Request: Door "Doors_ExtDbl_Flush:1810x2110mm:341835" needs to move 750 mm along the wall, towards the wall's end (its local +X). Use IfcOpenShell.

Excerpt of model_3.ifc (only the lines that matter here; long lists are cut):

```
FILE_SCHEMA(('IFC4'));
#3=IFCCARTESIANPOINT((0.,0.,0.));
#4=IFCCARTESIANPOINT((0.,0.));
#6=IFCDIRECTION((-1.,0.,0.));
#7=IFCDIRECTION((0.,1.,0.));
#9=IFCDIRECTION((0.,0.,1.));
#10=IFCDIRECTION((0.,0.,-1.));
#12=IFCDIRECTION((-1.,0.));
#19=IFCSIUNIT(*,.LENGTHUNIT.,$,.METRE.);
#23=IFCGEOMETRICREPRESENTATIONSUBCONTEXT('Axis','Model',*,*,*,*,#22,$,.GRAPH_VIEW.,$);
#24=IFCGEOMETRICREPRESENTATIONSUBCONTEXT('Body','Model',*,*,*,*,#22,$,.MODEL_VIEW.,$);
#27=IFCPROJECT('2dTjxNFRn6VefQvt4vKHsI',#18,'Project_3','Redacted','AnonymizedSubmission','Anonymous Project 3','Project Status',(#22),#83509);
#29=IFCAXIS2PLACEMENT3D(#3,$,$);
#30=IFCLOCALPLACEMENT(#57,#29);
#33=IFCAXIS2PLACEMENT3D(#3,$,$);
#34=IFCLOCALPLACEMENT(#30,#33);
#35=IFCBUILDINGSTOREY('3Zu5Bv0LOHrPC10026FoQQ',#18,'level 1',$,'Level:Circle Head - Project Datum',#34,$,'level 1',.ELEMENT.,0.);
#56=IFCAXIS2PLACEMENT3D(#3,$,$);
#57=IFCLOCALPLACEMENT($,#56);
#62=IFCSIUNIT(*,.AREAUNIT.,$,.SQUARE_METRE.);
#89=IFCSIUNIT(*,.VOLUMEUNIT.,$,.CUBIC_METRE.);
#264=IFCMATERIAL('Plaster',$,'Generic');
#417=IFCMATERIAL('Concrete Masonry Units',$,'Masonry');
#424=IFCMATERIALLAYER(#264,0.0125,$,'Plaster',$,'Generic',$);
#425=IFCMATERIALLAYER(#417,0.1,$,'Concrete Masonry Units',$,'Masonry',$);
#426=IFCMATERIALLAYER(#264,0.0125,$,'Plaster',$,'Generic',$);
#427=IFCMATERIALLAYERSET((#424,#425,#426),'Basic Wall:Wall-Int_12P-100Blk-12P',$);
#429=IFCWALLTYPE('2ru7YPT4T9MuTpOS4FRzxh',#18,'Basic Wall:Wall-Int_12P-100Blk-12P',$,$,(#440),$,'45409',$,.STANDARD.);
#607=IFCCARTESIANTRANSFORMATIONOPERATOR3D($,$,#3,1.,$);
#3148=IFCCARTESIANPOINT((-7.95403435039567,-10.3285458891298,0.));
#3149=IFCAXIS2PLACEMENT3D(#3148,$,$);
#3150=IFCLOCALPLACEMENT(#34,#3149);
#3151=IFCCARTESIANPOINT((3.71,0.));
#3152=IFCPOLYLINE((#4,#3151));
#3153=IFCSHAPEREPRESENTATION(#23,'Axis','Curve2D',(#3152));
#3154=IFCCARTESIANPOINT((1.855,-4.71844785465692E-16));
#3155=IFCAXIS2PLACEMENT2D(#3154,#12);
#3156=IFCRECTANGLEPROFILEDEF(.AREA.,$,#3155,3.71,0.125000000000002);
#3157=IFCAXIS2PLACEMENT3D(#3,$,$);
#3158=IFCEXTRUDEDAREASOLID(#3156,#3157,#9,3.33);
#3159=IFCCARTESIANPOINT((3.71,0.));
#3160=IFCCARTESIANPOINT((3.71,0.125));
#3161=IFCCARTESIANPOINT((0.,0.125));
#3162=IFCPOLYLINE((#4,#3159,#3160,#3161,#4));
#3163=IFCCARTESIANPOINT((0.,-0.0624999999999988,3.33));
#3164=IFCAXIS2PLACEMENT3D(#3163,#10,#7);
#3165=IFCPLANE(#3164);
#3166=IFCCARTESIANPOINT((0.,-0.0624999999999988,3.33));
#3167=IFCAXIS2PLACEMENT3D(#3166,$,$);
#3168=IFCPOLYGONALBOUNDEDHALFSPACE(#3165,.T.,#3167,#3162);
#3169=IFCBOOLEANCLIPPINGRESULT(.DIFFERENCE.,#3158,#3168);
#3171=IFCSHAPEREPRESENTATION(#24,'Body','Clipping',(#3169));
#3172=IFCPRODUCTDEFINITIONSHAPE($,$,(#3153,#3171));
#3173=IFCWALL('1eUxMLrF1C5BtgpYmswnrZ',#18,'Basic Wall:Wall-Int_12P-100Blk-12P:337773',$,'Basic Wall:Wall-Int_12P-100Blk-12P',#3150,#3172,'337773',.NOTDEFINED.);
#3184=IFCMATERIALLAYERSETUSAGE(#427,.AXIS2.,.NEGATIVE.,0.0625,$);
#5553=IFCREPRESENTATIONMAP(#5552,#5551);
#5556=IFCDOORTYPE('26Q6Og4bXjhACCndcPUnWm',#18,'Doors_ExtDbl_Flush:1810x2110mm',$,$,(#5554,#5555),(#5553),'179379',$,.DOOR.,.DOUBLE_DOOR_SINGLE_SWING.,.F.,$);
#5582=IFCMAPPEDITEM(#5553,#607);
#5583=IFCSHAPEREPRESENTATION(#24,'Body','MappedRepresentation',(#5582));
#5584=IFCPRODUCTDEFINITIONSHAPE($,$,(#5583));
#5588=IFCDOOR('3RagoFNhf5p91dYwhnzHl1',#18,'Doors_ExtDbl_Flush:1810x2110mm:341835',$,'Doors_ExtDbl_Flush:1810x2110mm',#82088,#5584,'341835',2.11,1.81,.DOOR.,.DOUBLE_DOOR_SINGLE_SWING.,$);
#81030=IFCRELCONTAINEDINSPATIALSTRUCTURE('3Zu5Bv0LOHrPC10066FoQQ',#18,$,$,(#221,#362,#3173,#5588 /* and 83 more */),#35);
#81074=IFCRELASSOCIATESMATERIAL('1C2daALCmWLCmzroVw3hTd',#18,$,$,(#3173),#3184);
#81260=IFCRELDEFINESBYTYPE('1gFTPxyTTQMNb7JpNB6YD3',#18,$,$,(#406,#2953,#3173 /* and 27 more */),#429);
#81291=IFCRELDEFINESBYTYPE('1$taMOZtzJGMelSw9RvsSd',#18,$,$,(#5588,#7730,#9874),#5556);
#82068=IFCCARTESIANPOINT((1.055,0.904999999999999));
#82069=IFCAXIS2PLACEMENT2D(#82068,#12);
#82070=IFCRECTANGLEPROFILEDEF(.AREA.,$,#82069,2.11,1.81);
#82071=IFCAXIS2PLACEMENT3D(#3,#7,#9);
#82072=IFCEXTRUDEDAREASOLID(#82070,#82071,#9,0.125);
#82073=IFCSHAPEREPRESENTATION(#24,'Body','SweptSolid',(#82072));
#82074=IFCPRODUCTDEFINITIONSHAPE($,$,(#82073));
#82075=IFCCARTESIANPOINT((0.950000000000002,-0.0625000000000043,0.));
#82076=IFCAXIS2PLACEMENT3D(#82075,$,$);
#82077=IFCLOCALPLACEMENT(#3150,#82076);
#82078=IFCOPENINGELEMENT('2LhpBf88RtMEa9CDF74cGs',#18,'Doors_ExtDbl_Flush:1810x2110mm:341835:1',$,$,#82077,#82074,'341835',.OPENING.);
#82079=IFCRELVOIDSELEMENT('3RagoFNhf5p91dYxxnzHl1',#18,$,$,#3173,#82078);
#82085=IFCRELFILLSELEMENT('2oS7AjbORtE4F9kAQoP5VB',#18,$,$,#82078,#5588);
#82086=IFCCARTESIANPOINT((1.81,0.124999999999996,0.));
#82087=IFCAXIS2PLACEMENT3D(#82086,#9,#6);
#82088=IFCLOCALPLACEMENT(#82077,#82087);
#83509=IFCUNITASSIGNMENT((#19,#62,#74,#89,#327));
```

```python
import ifcopenshell
import ifcopenshell.api.geometry
import ifcopenshell.util.placement
import ifcopenshell.util.unit

model = ifcopenshell.open("model_3.ifc")
unit_scale = ifcopenshell.util.unit.calculate_unit_scale(model)

door = model.by_guid("3RagoFNhf5p91dYwhnzHl1")
opening = door.FillsVoids[0].RelatingOpeningElement
wall = opening.VoidsElements[0].RelatingBuildingElement

wall_matrix = ifcopenshell.util.placement.get_local_placement(wall.ObjectPlacement)
shift = wall_matrix[:3, 0] * 0.75 / unit_scale
before = ifcopenshell.util.placement.get_local_placement(door.ObjectPlacement)[:3, 3].copy()

# The door is placed relative to its opening, so it follows when the opening moves.
matrix = ifcopenshell.util.placement.get_local_placement(opening.ObjectPlacement)
matrix[:3, 3] += shift
ifcopenshell.api.geometry.edit_object_placement(
    model, product=opening, matrix=matrix, is_si=False, should_transform_children=True
)

after = ifcopenshell.util.placement.get_local_placement(door.ObjectPlacement)[:3, 3]
print("door moved by", (after - before).round(3) + 0.0)

model.write("model_3_updated.ifc")
```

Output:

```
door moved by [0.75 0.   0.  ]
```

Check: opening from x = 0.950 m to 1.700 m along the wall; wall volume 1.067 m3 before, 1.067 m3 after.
